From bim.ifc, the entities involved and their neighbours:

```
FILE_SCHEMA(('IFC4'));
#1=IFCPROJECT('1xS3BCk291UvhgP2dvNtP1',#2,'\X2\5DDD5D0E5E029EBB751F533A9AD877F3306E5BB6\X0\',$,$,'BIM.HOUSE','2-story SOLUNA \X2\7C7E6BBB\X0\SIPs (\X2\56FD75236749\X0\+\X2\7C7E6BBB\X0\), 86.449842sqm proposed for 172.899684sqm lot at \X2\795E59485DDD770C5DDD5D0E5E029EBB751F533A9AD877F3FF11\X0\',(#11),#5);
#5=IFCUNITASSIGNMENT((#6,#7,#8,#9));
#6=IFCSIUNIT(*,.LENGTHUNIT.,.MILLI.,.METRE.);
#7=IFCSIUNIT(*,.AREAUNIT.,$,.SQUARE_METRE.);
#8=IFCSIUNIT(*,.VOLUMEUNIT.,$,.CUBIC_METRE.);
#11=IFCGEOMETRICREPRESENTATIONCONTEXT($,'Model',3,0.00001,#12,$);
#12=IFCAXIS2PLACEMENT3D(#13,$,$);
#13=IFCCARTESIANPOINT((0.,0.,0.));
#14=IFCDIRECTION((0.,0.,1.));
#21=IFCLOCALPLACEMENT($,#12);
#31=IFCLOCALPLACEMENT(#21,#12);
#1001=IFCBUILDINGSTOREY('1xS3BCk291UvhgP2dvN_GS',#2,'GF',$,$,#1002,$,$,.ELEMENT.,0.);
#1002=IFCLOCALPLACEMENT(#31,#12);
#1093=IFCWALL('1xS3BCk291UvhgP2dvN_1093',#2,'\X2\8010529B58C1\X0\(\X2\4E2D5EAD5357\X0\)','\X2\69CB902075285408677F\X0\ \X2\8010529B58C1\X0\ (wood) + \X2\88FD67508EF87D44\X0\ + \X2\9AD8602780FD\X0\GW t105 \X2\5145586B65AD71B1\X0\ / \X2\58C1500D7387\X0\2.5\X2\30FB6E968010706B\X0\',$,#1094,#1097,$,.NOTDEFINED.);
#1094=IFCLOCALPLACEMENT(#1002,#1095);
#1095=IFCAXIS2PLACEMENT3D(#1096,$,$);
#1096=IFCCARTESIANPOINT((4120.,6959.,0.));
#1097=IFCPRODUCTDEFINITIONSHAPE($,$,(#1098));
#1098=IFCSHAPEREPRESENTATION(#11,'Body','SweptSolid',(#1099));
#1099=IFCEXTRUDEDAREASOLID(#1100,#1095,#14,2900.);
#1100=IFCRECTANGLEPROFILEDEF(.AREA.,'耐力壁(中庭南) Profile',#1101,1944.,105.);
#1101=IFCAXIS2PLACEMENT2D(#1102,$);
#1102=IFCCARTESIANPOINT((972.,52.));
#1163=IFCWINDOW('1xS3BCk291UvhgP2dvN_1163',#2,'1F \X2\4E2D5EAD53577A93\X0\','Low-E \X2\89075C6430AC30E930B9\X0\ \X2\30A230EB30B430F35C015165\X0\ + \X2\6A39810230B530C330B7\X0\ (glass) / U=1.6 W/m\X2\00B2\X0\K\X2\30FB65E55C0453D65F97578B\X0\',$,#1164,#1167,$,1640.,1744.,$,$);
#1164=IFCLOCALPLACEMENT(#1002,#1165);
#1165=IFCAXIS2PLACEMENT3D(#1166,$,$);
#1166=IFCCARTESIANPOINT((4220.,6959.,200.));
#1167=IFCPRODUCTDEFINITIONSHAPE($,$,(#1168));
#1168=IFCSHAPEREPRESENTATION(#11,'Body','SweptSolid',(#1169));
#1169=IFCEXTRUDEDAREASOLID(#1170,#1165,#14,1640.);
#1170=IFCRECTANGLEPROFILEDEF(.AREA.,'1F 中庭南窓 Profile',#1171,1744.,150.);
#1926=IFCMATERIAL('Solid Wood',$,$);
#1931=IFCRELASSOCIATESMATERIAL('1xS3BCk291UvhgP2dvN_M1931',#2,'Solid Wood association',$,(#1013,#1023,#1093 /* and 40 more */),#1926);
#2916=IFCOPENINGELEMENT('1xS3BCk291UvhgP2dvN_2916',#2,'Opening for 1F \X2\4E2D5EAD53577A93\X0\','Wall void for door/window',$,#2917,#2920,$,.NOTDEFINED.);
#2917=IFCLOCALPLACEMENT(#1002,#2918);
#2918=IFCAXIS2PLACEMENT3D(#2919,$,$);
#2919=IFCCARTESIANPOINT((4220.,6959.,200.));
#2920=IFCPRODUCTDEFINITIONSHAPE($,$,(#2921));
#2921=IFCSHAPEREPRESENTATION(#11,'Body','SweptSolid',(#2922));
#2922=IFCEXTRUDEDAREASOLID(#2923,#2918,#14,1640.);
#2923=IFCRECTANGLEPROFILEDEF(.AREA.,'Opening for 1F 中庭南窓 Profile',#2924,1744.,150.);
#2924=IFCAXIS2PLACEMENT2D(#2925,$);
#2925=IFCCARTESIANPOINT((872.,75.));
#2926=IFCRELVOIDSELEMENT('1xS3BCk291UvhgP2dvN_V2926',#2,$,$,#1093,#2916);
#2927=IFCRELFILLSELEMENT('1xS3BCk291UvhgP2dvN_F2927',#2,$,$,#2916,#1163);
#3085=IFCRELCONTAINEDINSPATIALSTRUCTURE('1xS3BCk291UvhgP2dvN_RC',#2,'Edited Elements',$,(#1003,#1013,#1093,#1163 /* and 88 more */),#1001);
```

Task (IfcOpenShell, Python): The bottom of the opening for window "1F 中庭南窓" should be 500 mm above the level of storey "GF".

```python
import numpy as np
import ifcopenshell
import ifcopenshell.api.geometry
import ifcopenshell.geom
import ifcopenshell.util.element
import ifcopenshell.util.placement
import ifcopenshell.util.shape
import ifcopenshell.util.unit

model = ifcopenshell.open("bim.ifc")
unit_scale = ifcopenshell.util.unit.calculate_unit_scale(model)

window = model.by_guid("1xS3BCk291UvhgP2dvN_1163")
opening = window.FillsVoids[0].RelatingOpeningElement
storey = ifcopenshell.util.element.get_container(window, ifc_class="IfcBuildingStorey")
level = ifcopenshell.util.placement.get_local_placement(storey.ObjectPlacement)[2, 3]

# The opening's origin need not be at the sill, so measure its lowest point.
shape = ifcopenshell.geom.create_shape(ifcopenshell.geom.settings(), opening)
bottom = ifcopenshell.util.shape.get_shape_bottom_elevation(shape, shape.geometry) / unit_scale
dz = level + 500.0 - bottom

shift = np.array([0.0, 0.0, dz])
# The window is not placed relative to its opening, so move both.
for product in (opening, window):
    matrix = ifcopenshell.util.placement.get_local_placement(product.ObjectPlacement)
    matrix[:3, 3] += shift
    ifcopenshell.api.geometry.edit_object_placement(model, product=product, matrix=matrix, is_si=False)

print(f"moved by {dz * unit_scale:+.3f} m")

model.write("bim_rev.ifc")
```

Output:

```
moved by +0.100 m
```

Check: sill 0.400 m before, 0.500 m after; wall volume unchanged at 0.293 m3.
